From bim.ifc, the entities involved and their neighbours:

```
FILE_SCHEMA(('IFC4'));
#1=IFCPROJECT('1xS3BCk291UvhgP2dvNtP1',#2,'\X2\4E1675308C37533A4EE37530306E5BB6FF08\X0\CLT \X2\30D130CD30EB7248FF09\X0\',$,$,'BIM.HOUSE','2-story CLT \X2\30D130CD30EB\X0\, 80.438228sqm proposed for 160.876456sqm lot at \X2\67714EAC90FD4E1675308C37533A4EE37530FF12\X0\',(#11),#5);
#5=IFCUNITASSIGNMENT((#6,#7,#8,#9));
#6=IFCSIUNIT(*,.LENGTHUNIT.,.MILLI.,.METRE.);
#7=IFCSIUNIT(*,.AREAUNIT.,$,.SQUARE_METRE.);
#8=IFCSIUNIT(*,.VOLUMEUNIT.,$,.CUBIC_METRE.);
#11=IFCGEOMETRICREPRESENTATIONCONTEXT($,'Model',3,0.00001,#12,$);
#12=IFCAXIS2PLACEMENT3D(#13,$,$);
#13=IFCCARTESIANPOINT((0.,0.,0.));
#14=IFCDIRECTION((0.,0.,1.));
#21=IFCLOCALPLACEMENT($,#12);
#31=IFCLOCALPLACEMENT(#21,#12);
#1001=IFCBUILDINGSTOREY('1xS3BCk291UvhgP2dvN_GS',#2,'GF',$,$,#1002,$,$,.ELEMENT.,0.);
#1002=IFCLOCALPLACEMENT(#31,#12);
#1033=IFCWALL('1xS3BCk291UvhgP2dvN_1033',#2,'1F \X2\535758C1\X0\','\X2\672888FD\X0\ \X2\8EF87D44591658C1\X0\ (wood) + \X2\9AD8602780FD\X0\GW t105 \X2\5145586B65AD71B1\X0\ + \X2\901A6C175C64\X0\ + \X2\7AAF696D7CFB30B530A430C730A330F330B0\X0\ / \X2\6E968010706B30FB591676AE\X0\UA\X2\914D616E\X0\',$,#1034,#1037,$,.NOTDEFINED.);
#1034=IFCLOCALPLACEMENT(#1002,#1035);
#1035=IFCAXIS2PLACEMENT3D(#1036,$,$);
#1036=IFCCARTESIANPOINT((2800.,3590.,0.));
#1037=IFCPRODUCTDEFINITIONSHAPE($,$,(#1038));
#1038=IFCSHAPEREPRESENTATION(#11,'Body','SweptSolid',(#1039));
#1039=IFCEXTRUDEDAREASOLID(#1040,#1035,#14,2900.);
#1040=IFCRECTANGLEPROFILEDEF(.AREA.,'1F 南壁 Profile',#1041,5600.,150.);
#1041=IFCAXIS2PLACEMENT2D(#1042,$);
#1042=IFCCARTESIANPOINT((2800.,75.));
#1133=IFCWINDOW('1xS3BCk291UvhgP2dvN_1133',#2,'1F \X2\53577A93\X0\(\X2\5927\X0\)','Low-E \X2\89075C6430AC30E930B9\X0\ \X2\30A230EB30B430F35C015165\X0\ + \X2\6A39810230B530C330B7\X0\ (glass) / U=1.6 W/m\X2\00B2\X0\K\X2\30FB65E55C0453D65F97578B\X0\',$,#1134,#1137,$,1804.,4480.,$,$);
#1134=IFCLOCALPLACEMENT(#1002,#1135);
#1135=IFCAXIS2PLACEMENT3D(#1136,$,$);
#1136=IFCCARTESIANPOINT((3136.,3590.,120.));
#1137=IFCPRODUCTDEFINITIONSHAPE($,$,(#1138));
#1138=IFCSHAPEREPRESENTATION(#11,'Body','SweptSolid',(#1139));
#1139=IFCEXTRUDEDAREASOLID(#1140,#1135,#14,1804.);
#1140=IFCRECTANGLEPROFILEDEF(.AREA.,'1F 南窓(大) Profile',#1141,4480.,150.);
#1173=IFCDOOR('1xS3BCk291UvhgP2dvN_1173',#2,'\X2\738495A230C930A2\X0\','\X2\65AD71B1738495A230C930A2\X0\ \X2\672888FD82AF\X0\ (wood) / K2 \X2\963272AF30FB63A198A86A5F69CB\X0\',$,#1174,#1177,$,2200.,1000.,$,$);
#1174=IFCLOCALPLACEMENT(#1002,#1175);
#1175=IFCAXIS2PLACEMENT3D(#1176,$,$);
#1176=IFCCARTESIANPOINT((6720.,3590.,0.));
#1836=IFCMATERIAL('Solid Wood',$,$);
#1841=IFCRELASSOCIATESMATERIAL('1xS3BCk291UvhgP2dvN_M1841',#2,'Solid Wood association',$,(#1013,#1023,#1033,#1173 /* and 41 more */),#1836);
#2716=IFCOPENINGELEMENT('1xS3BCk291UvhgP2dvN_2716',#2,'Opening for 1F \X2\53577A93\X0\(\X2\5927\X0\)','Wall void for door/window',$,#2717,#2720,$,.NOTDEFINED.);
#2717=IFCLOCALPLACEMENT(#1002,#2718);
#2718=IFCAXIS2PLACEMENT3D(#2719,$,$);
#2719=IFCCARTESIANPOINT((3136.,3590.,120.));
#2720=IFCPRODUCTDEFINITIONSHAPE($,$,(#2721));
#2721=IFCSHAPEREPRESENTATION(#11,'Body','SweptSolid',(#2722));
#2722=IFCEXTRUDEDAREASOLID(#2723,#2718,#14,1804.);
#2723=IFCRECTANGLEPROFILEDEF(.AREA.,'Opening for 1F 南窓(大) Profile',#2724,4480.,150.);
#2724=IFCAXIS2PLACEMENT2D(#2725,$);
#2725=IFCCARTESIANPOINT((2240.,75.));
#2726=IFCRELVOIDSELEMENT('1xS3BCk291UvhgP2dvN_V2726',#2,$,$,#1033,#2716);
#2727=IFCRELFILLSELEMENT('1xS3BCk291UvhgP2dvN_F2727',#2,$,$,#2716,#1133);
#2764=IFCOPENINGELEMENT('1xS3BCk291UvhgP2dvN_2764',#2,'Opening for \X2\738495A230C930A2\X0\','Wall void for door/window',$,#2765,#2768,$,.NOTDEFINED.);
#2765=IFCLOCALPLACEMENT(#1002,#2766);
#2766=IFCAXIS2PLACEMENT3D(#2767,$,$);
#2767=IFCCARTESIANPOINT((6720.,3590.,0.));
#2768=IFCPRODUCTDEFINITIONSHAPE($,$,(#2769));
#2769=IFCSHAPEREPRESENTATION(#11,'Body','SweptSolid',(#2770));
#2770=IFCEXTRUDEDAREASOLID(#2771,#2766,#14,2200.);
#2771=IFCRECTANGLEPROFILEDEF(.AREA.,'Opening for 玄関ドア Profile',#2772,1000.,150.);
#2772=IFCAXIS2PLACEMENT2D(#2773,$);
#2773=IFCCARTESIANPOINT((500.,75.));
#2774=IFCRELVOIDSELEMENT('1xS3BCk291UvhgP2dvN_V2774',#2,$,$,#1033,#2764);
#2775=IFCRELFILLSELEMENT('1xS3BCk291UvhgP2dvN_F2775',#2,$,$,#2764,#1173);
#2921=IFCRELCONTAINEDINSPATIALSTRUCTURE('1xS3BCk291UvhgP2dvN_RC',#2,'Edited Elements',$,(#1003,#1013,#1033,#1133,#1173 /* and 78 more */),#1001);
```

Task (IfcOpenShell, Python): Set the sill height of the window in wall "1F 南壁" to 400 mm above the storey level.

```python
import numpy as np
import ifcopenshell
import ifcopenshell.api.geometry
import ifcopenshell.geom
import ifcopenshell.util.element
import ifcopenshell.util.placement
import ifcopenshell.util.shape
import ifcopenshell.util.unit

model = ifcopenshell.open("bim.ifc")
unit_scale = ifcopenshell.util.unit.calculate_unit_scale(model)

window = model.by_id(1133)
opening = window.FillsVoids[0].RelatingOpeningElement
storey = ifcopenshell.util.element.get_container(window, ifc_class="IfcBuildingStorey")
level = ifcopenshell.util.placement.get_local_placement(storey.ObjectPlacement)[2, 3]

# The opening's origin need not be at the sill, so measure its lowest point.
shape = ifcopenshell.geom.create_shape(ifcopenshell.geom.settings(), opening)
bottom = ifcopenshell.util.shape.get_shape_bottom_elevation(shape, shape.geometry) / unit_scale
dz = level + 400.0 - bottom

shift = np.array([0.0, 0.0, dz])
# The window is not placed relative to its opening, so move both.
for product in (opening, window):
    matrix = ifcopenshell.util.placement.get_local_placement(product.ObjectPlacement)
    matrix[:3, 3] += shift
    ifcopenshell.api.geometry.edit_object_placement(model, product=product, matrix=matrix, is_si=False)

print(f"moved by {dz * unit_scale:+.3f} m")

model.write("bim-out.ifc")
```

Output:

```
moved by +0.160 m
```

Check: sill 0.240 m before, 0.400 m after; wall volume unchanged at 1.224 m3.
